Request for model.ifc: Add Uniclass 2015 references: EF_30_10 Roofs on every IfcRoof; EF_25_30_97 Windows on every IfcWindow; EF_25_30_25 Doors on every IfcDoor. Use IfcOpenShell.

First a look at what the model holds.

```python
import ifcopenshell

model = ifcopenshell.open("model.ifc")
print(model.schema)
print("classifications:", [c.Name for c in model.by_type("IfcClassification")])
for ifc_class in ("IfcDoor", "IfcRoof", "IfcStair", "IfcWall", "IfcWindow"):
    print(ifc_class, len(model.by_type(ifc_class)))
```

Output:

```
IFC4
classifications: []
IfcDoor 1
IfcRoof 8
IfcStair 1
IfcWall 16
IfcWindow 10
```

```python
import ifcopenshell
import ifcopenshell.api.classification

model = ifcopenshell.open("model.ifc")

system = ifcopenshell.api.classification.add_classification(model, classification="Uniclass 2015")

codes = {
    "IfcRoof": ("EF_30_10", "Roofs"),
    "IfcWindow": ("EF_25_30_97", "Windows"),
    "IfcDoor": ("EF_25_30_25", "Doors"),
}
for ifc_class, (code, name) in codes.items():
    products = model.by_type(ifc_class)
    ifcopenshell.api.classification.add_reference(
        model, products=products, classification=system, identification=code, name=name
    )
    print(code, len(products))

model.write("model-out.ifc")
```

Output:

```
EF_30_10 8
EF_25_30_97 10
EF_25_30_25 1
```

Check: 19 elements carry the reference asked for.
